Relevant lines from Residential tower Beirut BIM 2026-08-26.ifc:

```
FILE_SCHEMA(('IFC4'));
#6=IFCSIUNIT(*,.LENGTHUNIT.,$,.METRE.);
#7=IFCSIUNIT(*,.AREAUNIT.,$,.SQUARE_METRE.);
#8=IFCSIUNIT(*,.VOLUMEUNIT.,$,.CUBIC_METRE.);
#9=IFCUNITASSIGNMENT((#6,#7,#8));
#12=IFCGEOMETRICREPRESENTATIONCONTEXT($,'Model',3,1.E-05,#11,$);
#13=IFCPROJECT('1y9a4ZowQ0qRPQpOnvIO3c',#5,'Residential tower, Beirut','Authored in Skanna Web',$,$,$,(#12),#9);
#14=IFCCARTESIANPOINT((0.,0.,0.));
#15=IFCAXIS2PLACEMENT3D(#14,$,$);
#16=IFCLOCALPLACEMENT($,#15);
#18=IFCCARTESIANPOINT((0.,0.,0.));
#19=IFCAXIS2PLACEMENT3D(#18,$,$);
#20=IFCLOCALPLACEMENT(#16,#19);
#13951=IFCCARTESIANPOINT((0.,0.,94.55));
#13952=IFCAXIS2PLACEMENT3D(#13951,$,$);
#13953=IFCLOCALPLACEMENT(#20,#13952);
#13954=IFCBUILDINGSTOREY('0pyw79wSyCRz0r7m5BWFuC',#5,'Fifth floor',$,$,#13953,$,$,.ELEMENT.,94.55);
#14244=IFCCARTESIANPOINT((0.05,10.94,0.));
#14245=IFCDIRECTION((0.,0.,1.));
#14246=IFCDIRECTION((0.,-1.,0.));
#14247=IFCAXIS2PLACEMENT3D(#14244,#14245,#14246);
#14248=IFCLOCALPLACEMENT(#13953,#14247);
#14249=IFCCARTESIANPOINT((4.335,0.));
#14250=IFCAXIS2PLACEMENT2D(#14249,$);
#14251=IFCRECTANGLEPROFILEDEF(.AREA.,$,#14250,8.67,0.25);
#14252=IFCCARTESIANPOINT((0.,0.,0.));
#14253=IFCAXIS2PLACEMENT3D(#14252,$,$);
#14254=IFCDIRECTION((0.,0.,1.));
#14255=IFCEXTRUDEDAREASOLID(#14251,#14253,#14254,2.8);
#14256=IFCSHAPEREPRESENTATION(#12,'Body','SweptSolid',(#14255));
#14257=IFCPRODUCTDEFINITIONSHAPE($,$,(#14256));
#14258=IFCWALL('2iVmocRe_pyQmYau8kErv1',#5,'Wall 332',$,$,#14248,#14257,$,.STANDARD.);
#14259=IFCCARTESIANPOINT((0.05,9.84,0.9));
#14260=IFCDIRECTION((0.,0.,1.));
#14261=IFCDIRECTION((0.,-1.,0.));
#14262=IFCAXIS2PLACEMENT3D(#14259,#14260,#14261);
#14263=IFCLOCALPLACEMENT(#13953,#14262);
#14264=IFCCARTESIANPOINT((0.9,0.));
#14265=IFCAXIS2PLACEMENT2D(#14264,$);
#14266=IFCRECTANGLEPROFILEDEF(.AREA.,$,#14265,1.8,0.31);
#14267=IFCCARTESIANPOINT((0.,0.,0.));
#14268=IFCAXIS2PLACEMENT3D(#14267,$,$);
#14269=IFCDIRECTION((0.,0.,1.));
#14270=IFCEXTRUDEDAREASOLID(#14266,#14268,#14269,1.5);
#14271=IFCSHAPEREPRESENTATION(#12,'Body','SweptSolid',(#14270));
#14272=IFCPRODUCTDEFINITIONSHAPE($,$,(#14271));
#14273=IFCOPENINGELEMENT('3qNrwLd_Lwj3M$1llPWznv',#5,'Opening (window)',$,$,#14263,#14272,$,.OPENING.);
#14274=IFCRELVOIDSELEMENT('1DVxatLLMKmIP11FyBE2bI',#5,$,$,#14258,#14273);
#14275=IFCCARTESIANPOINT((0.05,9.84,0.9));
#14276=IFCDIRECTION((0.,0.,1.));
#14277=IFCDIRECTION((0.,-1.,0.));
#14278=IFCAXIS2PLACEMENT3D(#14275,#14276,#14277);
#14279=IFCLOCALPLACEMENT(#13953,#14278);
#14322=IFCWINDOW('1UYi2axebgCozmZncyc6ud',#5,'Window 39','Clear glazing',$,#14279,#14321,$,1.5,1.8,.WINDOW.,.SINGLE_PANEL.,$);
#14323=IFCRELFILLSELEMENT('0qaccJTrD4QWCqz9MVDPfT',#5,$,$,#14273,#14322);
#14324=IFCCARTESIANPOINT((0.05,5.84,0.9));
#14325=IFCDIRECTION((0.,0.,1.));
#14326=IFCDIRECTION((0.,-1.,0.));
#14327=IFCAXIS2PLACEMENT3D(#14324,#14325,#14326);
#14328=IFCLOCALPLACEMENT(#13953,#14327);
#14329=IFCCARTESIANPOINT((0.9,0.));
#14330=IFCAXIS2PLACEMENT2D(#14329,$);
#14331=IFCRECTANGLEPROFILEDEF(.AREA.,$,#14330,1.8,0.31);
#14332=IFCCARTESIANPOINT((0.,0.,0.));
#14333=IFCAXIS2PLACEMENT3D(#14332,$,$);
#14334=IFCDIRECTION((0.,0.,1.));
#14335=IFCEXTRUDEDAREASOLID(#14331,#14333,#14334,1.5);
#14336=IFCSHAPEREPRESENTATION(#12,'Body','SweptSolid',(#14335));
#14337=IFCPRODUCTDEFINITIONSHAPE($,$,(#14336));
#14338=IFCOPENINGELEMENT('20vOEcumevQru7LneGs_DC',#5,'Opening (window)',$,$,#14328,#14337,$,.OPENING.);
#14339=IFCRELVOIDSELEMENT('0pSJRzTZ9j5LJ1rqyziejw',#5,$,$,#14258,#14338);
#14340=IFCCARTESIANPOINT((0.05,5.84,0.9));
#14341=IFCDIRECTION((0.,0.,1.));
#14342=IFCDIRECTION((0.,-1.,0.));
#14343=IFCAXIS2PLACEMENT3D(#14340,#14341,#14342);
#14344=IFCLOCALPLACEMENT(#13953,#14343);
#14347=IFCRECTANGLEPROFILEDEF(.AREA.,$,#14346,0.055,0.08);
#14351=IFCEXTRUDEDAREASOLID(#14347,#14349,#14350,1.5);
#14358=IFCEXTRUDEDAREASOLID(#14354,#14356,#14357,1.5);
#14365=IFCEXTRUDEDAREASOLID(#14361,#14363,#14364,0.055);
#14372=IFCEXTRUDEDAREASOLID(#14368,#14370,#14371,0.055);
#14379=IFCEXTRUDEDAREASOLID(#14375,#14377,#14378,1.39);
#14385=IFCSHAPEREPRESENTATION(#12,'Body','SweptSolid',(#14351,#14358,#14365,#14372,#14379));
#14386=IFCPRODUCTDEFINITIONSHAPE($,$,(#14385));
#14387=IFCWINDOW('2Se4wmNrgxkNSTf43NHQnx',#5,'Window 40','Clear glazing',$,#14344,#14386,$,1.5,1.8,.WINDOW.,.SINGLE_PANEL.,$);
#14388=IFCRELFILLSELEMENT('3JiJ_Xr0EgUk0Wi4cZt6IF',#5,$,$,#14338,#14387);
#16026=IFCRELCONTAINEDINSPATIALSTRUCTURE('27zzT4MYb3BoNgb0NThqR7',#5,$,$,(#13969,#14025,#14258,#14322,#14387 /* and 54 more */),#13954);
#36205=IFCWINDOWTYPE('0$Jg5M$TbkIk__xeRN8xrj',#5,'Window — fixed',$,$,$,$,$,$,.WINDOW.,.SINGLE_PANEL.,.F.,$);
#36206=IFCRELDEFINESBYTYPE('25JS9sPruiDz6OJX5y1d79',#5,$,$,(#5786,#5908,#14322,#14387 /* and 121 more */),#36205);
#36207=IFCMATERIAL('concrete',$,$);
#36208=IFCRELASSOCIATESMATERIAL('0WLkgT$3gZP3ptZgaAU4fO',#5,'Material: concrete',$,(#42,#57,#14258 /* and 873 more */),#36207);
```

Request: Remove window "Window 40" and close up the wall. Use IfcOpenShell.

```python
import ifcopenshell
import ifcopenshell.api.feature
import ifcopenshell.api.root
import ifcopenshell.geom
import ifcopenshell.util.shape

model = ifcopenshell.open("Residential tower Beirut BIM 2026-08-26.ifc")
settings = ifcopenshell.geom.settings()


def volume(element):
    """Net volume in cubic metres, openings subtracted."""
    shape = ifcopenshell.geom.create_shape(settings, element)
    return ifcopenshell.util.shape.get_volume(shape.geometry)


window = model.by_id(14387)
opening = window.FillsVoids[0].RelatingOpeningElement
wall = opening.VoidsElements[0].RelatingBuildingElement
before = volume(wall)

ifcopenshell.api.root.remove_product(model, product=window)
ifcopenshell.api.feature.remove_feature(model, feature=opening)

after = volume(wall)

print(f"wall volume {before:.3f} -> {after:.3f} m3")

model.write("Residential tower Beirut BIM 2026-08-26_v2.ifc")
```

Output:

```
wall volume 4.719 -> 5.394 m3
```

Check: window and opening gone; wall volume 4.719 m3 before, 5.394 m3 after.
